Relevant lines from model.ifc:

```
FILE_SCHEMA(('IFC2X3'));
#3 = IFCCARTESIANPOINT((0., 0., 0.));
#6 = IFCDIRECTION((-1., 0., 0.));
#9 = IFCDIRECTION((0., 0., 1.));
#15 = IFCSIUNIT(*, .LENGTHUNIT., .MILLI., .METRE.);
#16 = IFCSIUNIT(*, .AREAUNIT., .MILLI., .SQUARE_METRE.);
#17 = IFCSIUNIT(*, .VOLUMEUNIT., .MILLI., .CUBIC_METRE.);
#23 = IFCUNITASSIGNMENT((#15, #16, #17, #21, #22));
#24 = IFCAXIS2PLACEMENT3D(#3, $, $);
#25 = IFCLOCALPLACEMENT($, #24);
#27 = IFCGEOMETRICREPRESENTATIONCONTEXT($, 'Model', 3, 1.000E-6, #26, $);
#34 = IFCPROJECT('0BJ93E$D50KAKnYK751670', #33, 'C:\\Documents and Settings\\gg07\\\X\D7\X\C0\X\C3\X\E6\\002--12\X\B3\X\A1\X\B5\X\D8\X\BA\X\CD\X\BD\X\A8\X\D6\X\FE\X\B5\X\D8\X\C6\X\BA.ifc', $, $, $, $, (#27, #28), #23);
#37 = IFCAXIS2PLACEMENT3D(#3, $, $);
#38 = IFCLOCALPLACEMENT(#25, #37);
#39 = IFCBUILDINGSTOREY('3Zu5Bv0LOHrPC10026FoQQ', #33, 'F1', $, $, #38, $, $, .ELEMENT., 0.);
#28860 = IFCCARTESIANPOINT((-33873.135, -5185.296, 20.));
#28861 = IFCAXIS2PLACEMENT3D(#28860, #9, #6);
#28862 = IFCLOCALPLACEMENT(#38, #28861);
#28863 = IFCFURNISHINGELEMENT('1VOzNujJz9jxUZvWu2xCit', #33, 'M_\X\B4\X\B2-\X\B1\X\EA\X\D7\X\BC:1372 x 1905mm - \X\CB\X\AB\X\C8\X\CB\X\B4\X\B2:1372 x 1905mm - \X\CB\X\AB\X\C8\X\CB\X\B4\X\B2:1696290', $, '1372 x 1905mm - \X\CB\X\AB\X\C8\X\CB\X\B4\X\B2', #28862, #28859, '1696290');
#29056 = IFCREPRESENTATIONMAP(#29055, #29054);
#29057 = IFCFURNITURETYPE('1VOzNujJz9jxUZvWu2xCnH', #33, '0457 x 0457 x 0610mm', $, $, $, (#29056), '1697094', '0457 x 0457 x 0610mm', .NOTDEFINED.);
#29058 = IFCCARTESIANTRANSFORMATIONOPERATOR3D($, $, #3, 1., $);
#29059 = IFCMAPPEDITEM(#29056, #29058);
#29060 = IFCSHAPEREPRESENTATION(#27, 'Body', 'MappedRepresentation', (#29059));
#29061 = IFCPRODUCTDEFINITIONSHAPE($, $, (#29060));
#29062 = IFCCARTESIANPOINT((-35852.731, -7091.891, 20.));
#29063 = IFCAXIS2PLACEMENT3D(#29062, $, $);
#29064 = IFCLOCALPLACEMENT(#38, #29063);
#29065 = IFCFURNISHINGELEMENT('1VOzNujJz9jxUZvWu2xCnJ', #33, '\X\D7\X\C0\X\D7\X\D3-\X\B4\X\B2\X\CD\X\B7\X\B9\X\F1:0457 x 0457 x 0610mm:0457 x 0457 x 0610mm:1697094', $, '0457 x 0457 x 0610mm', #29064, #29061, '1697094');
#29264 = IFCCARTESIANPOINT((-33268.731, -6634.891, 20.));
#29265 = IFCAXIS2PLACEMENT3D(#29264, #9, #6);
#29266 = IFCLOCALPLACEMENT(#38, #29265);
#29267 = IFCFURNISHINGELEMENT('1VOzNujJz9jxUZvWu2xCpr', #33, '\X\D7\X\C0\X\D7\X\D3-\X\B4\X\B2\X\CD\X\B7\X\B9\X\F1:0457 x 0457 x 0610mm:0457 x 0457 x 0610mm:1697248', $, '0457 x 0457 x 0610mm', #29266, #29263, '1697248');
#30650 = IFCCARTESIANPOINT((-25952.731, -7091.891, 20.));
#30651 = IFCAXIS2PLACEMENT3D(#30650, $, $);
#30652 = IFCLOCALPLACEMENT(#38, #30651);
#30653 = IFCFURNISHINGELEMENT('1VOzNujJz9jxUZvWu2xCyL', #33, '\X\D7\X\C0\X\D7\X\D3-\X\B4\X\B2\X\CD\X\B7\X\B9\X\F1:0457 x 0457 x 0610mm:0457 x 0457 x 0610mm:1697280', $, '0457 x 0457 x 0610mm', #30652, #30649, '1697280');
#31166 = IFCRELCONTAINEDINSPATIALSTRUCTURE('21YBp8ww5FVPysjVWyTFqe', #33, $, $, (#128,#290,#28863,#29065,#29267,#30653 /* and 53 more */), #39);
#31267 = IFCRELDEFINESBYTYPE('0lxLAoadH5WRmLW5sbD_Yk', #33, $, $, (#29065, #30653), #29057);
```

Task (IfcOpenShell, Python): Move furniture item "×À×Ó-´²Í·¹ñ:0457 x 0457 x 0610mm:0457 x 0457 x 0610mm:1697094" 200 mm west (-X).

```python
import ifcopenshell
import ifcopenshell.api.geometry
import ifcopenshell.util.placement

model = ifcopenshell.open("model.ifc")

item = model.by_id(29065)
matrix = ifcopenshell.util.placement.get_local_placement(item.ObjectPlacement)
matrix[0, 3] -= 200.0
ifcopenshell.api.geometry.edit_object_placement(model, product=item, matrix=matrix, is_si=False)

print(ifcopenshell.util.placement.get_local_placement(item.ObjectPlacement).round(3) + 0.0)

model.write("model_rev.ifc")
```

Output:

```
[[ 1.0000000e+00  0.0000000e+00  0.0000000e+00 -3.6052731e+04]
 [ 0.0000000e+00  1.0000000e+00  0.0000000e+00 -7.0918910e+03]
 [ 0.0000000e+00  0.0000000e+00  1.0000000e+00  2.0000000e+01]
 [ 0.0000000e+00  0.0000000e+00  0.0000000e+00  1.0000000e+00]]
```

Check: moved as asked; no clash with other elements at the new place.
